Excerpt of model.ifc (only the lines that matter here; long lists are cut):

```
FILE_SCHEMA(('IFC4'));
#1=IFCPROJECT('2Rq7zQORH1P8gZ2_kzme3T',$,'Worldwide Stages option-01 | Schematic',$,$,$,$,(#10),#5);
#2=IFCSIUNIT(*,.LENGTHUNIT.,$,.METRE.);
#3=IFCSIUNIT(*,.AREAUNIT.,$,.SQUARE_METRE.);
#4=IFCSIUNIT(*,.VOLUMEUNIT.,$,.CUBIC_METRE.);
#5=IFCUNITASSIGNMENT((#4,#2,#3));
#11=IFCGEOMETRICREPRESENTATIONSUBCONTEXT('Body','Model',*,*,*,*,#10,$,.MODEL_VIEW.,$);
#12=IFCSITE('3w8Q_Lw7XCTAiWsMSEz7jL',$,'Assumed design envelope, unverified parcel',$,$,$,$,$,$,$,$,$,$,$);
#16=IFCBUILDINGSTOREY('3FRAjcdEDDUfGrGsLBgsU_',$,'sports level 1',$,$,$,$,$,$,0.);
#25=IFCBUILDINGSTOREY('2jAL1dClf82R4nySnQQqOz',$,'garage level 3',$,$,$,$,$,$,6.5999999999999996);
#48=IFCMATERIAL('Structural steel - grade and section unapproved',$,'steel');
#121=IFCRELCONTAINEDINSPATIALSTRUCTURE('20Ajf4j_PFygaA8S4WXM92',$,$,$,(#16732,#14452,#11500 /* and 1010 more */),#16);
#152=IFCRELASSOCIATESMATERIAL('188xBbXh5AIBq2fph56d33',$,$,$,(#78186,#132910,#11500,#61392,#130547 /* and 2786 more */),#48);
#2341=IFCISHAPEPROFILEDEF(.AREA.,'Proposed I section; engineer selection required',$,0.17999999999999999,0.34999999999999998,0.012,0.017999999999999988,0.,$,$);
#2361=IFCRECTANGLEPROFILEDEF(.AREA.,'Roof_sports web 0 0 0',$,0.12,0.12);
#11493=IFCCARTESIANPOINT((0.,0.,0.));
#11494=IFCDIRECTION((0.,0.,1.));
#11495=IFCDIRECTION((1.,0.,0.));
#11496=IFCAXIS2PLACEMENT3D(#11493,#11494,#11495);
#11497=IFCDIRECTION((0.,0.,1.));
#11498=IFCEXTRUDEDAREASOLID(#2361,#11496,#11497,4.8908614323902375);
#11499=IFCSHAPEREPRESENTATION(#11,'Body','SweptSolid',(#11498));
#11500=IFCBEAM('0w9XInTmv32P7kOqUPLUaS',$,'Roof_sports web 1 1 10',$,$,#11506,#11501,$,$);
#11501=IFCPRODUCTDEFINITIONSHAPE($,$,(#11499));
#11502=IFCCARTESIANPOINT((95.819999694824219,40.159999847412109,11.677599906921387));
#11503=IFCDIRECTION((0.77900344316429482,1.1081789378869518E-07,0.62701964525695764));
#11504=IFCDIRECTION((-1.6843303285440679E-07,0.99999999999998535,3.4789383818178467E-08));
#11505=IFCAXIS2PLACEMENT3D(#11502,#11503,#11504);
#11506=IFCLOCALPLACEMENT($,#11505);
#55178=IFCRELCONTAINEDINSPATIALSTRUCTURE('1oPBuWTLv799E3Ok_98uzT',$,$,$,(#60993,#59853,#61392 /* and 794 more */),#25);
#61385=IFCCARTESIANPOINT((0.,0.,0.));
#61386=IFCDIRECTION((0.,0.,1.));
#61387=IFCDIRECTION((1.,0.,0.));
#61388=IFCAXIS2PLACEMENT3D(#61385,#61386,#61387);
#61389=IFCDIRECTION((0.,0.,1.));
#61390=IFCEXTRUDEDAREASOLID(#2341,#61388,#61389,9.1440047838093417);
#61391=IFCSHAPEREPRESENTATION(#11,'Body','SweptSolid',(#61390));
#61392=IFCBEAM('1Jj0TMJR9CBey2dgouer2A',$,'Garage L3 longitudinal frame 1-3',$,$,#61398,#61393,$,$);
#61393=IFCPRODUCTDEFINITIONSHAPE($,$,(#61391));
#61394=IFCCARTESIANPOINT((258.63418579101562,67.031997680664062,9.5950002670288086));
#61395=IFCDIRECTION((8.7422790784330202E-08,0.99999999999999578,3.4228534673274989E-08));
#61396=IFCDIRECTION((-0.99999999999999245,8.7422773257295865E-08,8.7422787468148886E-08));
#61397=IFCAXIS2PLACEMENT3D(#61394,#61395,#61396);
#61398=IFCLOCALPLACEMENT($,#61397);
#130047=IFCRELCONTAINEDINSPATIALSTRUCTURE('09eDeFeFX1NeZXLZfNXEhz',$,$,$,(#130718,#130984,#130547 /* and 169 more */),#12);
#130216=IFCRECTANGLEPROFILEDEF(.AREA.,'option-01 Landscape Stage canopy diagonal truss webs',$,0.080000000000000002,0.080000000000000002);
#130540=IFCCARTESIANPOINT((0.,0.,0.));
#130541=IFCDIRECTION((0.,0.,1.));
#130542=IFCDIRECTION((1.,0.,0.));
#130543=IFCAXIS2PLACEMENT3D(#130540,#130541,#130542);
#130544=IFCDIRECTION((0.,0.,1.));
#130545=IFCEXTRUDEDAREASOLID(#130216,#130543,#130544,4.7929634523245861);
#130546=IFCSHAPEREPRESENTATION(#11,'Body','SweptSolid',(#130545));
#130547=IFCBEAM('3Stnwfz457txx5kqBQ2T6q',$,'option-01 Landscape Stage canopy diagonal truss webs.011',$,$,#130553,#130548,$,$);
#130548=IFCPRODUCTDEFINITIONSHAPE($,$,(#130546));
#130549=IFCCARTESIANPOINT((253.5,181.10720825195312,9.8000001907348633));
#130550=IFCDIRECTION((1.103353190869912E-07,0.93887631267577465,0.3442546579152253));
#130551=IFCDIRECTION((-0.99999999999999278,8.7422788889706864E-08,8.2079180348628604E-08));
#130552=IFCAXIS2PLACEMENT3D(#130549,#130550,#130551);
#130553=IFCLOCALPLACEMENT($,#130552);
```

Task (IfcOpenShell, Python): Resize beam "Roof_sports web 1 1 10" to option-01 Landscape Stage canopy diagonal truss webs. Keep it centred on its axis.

```python
import ifcopenshell
import ifcopenshell.util.element
import ifcopenshell.util.representation

model = ifcopenshell.open("model.ifc")

member = model.by_id(11500)
source = next(p for p in model.by_type("IfcRectangleProfileDef") if p.ProfileName == "option-01 Landscape Stage canopy diagonal truss webs")

body = ifcopenshell.util.representation.get_representation(member, "Model", "Body")
solid = body.Items[0]
old_profile = solid.SweptArea

# Copy the section's sizes but keep this member's own profile position.
profile = ifcopenshell.util.element.copy(model, source)
profile.Position = old_profile.Position
solid.SweptArea = profile
if not model.get_total_inverses(old_profile):
    ifcopenshell.util.element.remove_deep2(model, old_profile)

print(solid.SweptArea)

model.write("model_edited.ifc")
```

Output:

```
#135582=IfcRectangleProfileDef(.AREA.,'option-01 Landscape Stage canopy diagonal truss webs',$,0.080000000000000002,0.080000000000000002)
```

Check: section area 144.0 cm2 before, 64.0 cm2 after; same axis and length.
